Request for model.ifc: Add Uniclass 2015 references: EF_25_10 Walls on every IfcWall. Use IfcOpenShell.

First a look at what the model holds.

```python
import ifcopenshell

model = ifcopenshell.open("model.ifc")
print(model.schema)
print("classifications:", [c.Name for c in model.by_type("IfcClassification")])
for ifc_class in ("IfcDoor", "IfcRoof", "IfcStair", "IfcWall", "IfcWindow"):
    print(ifc_class, len(model.by_type(ifc_class)))
```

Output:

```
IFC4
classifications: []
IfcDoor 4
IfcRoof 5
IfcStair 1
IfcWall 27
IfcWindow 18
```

```python
import ifcopenshell
import ifcopenshell.api.classification

model = ifcopenshell.open("model.ifc")

system = ifcopenshell.api.classification.add_classification(model, classification="Uniclass 2015")

codes = {
    "IfcWall": ("EF_25_10", "Walls"),
}
for ifc_class, (code, name) in codes.items():
    products = model.by_type(ifc_class)
    ifcopenshell.api.classification.add_reference(
        model, products=products, classification=system, identification=code, name=name
    )
    print(code, len(products))

model.write("model_v2.ifc")
```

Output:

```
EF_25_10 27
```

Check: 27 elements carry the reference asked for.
